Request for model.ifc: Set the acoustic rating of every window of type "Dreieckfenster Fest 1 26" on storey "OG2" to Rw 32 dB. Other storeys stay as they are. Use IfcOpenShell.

First a look at what the model holds.

```python
import ifcopenshell
import ifcopenshell.util.element

model = ifcopenshell.open("model.ifc")
print(model.schema)
storey = next(s for s in model.by_type("IfcBuildingStorey") if s.Name == "OG2")
windows = [e for e in ifcopenshell.util.element.get_decomposition(storey) if e.is_a("IfcWindow")]
seen = {}
for e in windows:
    element_type = ifcopenshell.util.element.get_type(e)
    key = (element_type.Name if element_type != e and element_type else None, ifcopenshell.util.element.get_pset(e, "Pset_WindowCommon", "AcousticRating"))
    seen[key] = seen.get(key, 0) + 1
for (name, value), count in sorted(seen.items(), key=str):
    print(count, "x", name, "|", value)
```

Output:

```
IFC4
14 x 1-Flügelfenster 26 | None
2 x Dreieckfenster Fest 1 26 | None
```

```python
import ifcopenshell
import ifcopenshell.api.pset
import ifcopenshell.util.element

model = ifcopenshell.open("model.ifc")

storey = next(s for s in model.by_type("IfcBuildingStorey") if s.Name == "OG2")
windows = [e for e in ifcopenshell.util.element.get_decomposition(storey) if e.is_a("IfcWindow")]

count = 0
for e in windows:
    element_type = ifcopenshell.util.element.get_type(e)
    if element_type in (None, e) or element_type.Name != "Dreieckfenster Fest 1 26":
        continue
    # add_pset returns the element's existing set when there is one.
    pset = ifcopenshell.api.pset.add_pset(model, product=e, name="Pset_WindowCommon")
    ifcopenshell.api.pset.edit_pset(model, pset=pset, properties={"AcousticRating": "Rw 32 dB"})
    count += 1

print(count, "windows updated")

model.write("model_updated.ifc")
```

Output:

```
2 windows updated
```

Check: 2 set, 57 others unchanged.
